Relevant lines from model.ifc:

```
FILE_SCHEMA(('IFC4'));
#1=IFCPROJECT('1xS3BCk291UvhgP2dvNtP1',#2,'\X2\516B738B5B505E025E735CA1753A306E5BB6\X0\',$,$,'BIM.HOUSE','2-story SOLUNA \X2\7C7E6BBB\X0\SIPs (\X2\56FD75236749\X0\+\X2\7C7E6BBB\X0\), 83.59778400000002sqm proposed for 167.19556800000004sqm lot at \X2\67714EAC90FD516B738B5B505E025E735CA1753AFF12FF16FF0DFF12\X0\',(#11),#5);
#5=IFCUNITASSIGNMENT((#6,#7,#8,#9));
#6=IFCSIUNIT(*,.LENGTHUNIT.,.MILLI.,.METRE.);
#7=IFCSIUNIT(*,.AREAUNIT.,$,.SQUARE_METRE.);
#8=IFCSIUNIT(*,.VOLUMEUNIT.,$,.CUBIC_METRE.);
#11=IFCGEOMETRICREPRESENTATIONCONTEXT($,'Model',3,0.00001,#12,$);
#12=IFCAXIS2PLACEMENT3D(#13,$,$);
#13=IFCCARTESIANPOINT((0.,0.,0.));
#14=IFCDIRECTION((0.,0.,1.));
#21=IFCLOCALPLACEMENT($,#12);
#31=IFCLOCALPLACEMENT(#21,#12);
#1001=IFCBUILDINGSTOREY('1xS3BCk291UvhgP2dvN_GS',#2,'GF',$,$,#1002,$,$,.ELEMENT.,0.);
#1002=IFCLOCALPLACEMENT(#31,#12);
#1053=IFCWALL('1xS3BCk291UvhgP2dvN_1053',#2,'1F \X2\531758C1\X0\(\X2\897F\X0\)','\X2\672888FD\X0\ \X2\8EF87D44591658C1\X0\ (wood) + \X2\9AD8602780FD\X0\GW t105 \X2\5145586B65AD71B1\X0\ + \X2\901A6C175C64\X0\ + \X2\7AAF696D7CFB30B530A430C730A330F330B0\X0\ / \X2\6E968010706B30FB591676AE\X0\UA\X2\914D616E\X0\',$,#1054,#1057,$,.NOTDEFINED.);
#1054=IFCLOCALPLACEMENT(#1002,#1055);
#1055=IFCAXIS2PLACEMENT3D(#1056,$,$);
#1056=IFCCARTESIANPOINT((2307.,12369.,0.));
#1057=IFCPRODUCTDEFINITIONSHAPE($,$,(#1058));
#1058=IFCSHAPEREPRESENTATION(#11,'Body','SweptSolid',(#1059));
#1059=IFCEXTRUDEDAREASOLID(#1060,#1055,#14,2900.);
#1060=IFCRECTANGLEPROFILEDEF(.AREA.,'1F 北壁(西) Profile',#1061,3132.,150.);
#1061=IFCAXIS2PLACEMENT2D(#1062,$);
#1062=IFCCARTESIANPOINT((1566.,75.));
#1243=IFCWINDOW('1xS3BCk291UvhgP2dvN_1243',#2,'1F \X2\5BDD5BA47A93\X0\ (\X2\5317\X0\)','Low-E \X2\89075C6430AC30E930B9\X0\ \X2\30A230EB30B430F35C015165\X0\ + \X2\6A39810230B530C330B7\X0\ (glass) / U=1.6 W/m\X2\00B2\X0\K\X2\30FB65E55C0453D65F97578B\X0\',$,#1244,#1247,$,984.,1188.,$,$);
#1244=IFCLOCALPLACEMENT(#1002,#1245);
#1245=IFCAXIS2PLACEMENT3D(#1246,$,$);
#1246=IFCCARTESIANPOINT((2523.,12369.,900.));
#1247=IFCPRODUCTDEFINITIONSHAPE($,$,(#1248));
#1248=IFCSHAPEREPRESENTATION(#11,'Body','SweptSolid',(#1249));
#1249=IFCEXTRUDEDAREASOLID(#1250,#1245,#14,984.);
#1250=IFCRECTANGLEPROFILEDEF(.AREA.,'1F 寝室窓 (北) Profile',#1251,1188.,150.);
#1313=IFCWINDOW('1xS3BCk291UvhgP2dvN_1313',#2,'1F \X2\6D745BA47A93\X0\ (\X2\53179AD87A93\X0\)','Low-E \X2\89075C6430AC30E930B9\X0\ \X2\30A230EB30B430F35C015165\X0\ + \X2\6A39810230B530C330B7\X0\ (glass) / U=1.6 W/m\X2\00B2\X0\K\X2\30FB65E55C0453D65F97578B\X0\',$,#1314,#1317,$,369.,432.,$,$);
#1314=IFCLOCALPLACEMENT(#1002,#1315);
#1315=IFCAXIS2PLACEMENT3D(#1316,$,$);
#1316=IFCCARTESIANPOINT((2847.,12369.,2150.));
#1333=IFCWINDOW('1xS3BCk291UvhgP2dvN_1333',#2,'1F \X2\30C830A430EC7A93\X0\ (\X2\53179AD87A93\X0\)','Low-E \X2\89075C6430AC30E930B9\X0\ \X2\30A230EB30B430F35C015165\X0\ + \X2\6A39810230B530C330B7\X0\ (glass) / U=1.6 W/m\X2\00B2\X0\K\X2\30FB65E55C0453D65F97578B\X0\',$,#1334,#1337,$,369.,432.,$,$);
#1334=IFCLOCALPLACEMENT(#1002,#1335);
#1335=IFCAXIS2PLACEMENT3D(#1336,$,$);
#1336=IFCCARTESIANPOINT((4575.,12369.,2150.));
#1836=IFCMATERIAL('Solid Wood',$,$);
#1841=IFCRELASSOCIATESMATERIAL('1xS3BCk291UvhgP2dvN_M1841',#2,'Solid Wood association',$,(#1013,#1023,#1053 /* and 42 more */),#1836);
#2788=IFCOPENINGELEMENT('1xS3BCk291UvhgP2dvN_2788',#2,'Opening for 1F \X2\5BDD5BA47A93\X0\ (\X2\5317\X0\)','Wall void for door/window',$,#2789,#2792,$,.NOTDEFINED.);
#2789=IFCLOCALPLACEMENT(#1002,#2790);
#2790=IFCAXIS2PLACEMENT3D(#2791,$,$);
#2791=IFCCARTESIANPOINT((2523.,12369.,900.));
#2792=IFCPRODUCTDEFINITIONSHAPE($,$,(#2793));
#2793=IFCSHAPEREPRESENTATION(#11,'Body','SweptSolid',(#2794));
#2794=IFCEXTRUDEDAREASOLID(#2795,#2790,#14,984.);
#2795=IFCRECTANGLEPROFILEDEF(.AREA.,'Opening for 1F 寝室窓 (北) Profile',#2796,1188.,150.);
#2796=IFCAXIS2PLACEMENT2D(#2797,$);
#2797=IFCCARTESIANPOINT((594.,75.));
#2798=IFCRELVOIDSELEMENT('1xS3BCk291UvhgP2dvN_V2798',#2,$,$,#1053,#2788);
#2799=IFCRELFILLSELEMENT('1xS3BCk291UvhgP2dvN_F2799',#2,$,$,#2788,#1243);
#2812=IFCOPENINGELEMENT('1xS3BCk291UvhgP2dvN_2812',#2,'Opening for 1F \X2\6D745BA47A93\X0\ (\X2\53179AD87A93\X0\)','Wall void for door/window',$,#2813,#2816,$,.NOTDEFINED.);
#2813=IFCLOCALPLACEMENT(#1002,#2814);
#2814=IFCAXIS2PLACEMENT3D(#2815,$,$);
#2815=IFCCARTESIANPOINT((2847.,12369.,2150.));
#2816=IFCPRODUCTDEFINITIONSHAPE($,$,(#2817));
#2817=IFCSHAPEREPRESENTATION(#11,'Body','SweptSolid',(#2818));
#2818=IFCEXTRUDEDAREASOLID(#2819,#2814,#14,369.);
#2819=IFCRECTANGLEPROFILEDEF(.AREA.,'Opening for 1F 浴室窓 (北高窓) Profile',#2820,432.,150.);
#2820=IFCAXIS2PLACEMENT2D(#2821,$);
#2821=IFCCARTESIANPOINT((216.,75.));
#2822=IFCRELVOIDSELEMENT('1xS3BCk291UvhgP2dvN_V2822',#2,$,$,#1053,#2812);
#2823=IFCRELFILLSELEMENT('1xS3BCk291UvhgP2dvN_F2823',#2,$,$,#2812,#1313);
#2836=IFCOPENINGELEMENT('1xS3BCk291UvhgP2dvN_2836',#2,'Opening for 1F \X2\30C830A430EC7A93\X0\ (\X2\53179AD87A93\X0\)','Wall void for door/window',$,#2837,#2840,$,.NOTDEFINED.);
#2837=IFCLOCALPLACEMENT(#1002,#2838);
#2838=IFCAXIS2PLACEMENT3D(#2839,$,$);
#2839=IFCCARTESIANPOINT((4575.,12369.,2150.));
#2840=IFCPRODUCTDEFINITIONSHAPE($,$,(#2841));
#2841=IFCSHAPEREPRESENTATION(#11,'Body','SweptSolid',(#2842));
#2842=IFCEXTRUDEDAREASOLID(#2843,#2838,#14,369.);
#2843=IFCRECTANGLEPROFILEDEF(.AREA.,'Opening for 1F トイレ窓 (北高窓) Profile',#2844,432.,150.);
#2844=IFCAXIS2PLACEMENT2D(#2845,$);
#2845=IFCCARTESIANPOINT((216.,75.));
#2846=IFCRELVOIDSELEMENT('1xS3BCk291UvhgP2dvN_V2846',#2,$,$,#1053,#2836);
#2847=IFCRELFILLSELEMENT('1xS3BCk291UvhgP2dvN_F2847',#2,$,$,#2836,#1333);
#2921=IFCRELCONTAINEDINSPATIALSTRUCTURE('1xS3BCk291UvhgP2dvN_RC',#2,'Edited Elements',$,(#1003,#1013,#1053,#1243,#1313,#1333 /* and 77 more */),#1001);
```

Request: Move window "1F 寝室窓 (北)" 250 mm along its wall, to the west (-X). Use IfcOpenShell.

```python
import ifcopenshell
import ifcopenshell.api.geometry
import ifcopenshell.util.placement
import ifcopenshell.util.unit

model = ifcopenshell.open("model.ifc")
unit_scale = ifcopenshell.util.unit.calculate_unit_scale(model)

window = model.by_guid("1xS3BCk291UvhgP2dvN_1243")
opening = window.FillsVoids[0].RelatingOpeningElement
wall = opening.VoidsElements[0].RelatingBuildingElement

wall_matrix = ifcopenshell.util.placement.get_local_placement(wall.ObjectPlacement)
shift = wall_matrix[:3, 0] * -0.25 / unit_scale
before = ifcopenshell.util.placement.get_local_placement(window.ObjectPlacement)[:3, 3].copy()

# The window is not placed relative to its opening, so move both.
for product in (opening, window):
    matrix = ifcopenshell.util.placement.get_local_placement(product.ObjectPlacement)
    matrix[:3, 3] += shift
    ifcopenshell.api.geometry.edit_object_placement(model, product=product, matrix=matrix, is_si=False)

after = ifcopenshell.util.placement.get_local_placement(window.ObjectPlacement)[:3, 3]
print("window moved by", (after - before).round(3) + 0.0)

model.write("model_v2.ifc")
```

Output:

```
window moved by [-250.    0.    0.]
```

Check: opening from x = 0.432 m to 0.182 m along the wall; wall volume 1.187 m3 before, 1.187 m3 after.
